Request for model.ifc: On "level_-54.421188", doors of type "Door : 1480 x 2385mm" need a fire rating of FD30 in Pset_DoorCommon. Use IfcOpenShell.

First a look at what the model holds.

```python
import ifcopenshell
import ifcopenshell.util.element

model = ifcopenshell.open("model.ifc")
print(model.schema)
storey = next(s for s in model.by_type("IfcBuildingStorey") if s.Name == "level_-54.421188")
doors = [e for e in ifcopenshell.util.element.get_decomposition(storey) if e.is_a("IfcDoor")]
seen = {}
for e in doors:
    element_type = ifcopenshell.util.element.get_type(e)
    key = (element_type.Name if element_type != e and element_type else None, ifcopenshell.util.element.get_pset(e, "Pset_DoorCommon", "FireRating"))
    seen[key] = seen.get(key, 0) + 1
for (name, value), count in sorted(seen.items(), key=str):
    print(count, "x", name, "|", value)
```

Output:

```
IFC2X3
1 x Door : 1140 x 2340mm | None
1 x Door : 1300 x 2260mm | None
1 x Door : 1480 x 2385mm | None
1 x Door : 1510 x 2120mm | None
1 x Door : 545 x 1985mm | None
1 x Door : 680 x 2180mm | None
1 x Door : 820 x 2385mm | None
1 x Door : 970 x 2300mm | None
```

```python
import ifcopenshell
import ifcopenshell.api.pset
import ifcopenshell.util.element

model = ifcopenshell.open("model.ifc")

storey = next(s for s in model.by_type("IfcBuildingStorey") if s.Name == "level_-54.421188")
doors = [e for e in ifcopenshell.util.element.get_decomposition(storey) if e.is_a("IfcDoor")]

count = 0
for e in doors:
    element_type = ifcopenshell.util.element.get_type(e)
    if element_type in (None, e) or element_type.Name != "Door : 1480 x 2385mm":
        continue
    # add_pset returns the element's existing set when there is one.
    pset = ifcopenshell.api.pset.add_pset(model, product=e, name="Pset_DoorCommon")
    ifcopenshell.api.pset.edit_pset(model, pset=pset, properties={"FireRating": "FD30"})
    count += 1

print(count, "doors updated")

model.write("model-out.ifc")
```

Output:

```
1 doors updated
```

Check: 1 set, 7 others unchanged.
